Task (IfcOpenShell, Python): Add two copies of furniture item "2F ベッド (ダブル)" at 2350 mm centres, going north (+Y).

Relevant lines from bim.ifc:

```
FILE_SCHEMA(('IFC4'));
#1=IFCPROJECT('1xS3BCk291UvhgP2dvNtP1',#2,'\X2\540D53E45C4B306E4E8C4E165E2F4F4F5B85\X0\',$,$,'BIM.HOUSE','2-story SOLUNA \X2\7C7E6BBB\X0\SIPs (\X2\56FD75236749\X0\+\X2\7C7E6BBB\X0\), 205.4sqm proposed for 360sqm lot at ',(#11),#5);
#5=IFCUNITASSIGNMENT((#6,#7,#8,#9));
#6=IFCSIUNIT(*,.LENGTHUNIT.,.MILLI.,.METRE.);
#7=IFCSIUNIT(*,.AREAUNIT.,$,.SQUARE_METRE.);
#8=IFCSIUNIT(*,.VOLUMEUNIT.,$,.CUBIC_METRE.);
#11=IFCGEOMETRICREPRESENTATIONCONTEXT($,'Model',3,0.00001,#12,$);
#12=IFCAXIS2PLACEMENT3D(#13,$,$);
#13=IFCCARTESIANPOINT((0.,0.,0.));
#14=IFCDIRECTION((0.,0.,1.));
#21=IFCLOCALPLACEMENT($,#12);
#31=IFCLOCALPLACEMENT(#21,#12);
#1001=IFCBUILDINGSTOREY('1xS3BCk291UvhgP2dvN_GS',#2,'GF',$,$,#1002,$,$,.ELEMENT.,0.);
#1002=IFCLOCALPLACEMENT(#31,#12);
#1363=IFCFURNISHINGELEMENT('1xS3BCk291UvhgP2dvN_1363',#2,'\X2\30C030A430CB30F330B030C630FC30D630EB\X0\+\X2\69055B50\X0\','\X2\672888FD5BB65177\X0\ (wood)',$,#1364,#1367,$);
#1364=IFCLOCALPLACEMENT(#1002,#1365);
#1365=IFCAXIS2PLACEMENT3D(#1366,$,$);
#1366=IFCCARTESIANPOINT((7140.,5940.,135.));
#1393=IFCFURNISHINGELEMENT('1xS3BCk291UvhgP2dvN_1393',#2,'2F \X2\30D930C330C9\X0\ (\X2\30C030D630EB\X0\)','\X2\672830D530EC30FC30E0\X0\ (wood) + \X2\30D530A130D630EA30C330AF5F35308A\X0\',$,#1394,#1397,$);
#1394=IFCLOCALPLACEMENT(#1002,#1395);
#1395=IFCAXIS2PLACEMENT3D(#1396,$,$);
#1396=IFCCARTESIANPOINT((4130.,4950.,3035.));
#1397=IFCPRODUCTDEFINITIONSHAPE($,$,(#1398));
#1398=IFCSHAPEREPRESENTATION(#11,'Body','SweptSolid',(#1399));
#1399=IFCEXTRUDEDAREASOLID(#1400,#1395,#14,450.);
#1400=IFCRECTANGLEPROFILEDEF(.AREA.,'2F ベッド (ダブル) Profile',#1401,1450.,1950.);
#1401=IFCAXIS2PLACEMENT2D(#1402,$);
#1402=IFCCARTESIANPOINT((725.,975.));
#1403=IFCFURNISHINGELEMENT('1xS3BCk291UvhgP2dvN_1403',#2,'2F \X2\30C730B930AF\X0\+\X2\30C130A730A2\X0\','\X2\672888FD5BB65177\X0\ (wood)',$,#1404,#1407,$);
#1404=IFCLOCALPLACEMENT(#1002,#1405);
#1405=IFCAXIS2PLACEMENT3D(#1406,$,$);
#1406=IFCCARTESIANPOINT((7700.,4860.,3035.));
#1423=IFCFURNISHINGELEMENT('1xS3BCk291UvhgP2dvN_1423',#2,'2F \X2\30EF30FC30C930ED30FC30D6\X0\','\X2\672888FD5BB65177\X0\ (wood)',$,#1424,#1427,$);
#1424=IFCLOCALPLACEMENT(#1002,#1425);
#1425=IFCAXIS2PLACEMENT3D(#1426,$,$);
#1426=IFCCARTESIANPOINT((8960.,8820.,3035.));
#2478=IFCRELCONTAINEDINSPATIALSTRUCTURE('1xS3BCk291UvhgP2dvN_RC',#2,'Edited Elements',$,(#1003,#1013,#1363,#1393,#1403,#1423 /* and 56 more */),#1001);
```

```python
import numpy as np
import ifcopenshell
import ifcopenshell.api.geometry
import ifcopenshell.api.root
import ifcopenshell.util.element
import ifcopenshell.util.placement

model = ifcopenshell.open("bim.ifc")


def reuse_history(source, copy):
    """copy_class also copies each property set's owner history, people and application; keep the originals."""
    for rel in copy.IsDefinedBy:
        if rel.is_a("IfcRelDefinesByProperties") and (history := rel.RelatingPropertyDefinition.OwnerHistory):
            rel.RelatingPropertyDefinition.OwnerHistory = source.OwnerHistory
            ifcopenshell.util.element.remove_deep2(model, history)


source = model.by_id(1393)
base = ifcopenshell.util.placement.get_local_placement(source.ObjectPlacement)
step = np.array([0.0, 1.0, 0.0]) * 2350.0

for i in range(1, 3):
    copy = ifcopenshell.api.root.copy_class(model, product=source)
    copy.Representation = ifcopenshell.util.element.copy_deep(
        model, source.Representation, exclude=["IfcGeometricRepresentationContext", "IfcRepresentationMap"]
    )
    reuse_history(source, copy)
    matrix = base.copy()
    matrix[:3, 3] += i * step
    print("added at", matrix[:3, 3].round(3) + 0.0)
    ifcopenshell.api.geometry.edit_object_placement(model, product=copy, matrix=matrix, is_si=False)

model.write("bim_v2.ifc")
```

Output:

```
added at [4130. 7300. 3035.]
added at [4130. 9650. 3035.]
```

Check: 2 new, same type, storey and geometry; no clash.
